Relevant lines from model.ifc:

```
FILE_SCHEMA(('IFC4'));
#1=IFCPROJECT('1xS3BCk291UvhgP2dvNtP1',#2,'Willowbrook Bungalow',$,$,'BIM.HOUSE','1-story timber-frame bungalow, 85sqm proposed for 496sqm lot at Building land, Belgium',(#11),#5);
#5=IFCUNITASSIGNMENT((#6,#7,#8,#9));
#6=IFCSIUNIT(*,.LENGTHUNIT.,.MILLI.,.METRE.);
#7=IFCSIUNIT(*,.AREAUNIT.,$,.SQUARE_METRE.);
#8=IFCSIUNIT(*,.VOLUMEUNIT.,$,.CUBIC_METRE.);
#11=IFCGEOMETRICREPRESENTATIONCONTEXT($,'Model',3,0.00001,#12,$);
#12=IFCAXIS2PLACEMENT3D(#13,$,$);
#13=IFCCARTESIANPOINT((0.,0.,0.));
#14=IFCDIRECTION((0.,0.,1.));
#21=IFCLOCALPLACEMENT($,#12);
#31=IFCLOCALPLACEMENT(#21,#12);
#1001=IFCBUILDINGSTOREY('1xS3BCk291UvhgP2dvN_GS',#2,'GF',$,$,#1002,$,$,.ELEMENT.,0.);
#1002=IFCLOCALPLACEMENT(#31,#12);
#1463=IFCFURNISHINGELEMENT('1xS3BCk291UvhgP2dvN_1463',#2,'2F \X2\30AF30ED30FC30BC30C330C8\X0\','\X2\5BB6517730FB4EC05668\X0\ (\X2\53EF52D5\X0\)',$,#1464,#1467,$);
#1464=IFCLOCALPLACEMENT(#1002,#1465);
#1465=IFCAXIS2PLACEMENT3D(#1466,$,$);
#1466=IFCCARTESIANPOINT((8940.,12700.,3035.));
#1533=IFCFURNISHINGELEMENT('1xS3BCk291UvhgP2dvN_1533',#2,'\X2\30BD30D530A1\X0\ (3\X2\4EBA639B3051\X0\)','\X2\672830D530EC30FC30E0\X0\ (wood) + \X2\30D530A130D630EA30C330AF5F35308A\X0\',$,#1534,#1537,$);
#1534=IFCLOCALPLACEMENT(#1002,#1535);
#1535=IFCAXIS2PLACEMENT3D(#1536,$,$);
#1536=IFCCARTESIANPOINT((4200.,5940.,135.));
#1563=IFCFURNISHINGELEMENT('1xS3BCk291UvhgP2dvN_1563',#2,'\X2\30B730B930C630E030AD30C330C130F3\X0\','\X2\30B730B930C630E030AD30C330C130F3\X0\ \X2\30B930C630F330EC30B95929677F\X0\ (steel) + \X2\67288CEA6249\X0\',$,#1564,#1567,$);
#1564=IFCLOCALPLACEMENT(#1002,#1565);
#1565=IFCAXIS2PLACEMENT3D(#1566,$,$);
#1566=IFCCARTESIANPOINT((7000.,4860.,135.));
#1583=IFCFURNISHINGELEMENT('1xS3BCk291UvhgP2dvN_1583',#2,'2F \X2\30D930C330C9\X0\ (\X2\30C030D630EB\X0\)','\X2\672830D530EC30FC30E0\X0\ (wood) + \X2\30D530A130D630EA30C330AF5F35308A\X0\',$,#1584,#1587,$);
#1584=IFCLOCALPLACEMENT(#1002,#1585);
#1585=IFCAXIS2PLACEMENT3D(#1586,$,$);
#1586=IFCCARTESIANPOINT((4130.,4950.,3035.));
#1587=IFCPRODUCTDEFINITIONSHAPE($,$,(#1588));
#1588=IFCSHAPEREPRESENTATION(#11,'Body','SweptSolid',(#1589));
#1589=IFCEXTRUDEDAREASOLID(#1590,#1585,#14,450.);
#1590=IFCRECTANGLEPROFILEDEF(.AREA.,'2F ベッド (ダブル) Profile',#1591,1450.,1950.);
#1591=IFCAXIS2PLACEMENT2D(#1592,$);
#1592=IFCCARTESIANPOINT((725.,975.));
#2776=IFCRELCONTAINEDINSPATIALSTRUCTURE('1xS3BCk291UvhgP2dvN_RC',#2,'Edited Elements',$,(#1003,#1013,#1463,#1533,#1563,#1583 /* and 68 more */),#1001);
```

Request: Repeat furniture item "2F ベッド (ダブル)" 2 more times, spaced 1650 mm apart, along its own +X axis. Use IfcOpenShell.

```python
import ifcopenshell
import ifcopenshell.api.geometry
import ifcopenshell.api.root
import ifcopenshell.util.element
import ifcopenshell.util.placement
import ifcopenshell.util.unit

model = ifcopenshell.open("model.ifc")
unit_scale = ifcopenshell.util.unit.calculate_unit_scale(model)


def reuse_history(source, copy):
    """copy_class also copies each property set's owner history, people and application; keep the originals."""
    for rel in copy.IsDefinedBy:
        if rel.is_a("IfcRelDefinesByProperties") and (history := rel.RelatingPropertyDefinition.OwnerHistory):
            rel.RelatingPropertyDefinition.OwnerHistory = source.OwnerHistory
            ifcopenshell.util.element.remove_deep2(model, history)


source = model.by_id(1583)
base = ifcopenshell.util.placement.get_local_placement(source.ObjectPlacement)
step = base[:3, 0] * 1.65 / unit_scale

for i in range(1, 3):
    copy = ifcopenshell.api.root.copy_class(model, product=source)
    copy.Representation = ifcopenshell.util.element.copy_deep(
        model, source.Representation, exclude=["IfcGeometricRepresentationContext", "IfcRepresentationMap"]
    )
    reuse_history(source, copy)
    matrix = base.copy()
    matrix[:3, 3] += i * step
    print("added at", matrix[:3, 3].round(3) + 0.0)
    ifcopenshell.api.geometry.edit_object_placement(model, product=copy, matrix=matrix, is_si=False)

model.write("model-out.ifc")
```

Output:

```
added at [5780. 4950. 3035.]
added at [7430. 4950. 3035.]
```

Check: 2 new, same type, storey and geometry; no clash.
